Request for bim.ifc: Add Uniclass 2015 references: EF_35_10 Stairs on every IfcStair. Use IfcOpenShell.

First a look at what the model holds.

```python
import ifcopenshell

model = ifcopenshell.open("bim.ifc")
print(model.schema)
print("classifications:", [c.Name for c in model.by_type("IfcClassification")])
for ifc_class in ("IfcDoor", "IfcRoof", "IfcStair", "IfcWall", "IfcWindow"):
    print(ifc_class, len(model.by_type(ifc_class)))
```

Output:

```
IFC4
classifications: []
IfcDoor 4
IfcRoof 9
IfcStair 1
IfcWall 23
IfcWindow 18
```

```python
import ifcopenshell
import ifcopenshell.api.classification

model = ifcopenshell.open("bim.ifc")

system = ifcopenshell.api.classification.add_classification(model, classification="Uniclass 2015")

codes = {
    "IfcStair": ("EF_35_10", "Stairs"),
}
for ifc_class, (code, name) in codes.items():
    products = model.by_type(ifc_class)
    ifcopenshell.api.classification.add_reference(
        model, products=products, classification=system, identification=code, name=name
    )
    print(code, len(products))

model.write("bim-out.ifc")
```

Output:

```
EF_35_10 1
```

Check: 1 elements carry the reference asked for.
